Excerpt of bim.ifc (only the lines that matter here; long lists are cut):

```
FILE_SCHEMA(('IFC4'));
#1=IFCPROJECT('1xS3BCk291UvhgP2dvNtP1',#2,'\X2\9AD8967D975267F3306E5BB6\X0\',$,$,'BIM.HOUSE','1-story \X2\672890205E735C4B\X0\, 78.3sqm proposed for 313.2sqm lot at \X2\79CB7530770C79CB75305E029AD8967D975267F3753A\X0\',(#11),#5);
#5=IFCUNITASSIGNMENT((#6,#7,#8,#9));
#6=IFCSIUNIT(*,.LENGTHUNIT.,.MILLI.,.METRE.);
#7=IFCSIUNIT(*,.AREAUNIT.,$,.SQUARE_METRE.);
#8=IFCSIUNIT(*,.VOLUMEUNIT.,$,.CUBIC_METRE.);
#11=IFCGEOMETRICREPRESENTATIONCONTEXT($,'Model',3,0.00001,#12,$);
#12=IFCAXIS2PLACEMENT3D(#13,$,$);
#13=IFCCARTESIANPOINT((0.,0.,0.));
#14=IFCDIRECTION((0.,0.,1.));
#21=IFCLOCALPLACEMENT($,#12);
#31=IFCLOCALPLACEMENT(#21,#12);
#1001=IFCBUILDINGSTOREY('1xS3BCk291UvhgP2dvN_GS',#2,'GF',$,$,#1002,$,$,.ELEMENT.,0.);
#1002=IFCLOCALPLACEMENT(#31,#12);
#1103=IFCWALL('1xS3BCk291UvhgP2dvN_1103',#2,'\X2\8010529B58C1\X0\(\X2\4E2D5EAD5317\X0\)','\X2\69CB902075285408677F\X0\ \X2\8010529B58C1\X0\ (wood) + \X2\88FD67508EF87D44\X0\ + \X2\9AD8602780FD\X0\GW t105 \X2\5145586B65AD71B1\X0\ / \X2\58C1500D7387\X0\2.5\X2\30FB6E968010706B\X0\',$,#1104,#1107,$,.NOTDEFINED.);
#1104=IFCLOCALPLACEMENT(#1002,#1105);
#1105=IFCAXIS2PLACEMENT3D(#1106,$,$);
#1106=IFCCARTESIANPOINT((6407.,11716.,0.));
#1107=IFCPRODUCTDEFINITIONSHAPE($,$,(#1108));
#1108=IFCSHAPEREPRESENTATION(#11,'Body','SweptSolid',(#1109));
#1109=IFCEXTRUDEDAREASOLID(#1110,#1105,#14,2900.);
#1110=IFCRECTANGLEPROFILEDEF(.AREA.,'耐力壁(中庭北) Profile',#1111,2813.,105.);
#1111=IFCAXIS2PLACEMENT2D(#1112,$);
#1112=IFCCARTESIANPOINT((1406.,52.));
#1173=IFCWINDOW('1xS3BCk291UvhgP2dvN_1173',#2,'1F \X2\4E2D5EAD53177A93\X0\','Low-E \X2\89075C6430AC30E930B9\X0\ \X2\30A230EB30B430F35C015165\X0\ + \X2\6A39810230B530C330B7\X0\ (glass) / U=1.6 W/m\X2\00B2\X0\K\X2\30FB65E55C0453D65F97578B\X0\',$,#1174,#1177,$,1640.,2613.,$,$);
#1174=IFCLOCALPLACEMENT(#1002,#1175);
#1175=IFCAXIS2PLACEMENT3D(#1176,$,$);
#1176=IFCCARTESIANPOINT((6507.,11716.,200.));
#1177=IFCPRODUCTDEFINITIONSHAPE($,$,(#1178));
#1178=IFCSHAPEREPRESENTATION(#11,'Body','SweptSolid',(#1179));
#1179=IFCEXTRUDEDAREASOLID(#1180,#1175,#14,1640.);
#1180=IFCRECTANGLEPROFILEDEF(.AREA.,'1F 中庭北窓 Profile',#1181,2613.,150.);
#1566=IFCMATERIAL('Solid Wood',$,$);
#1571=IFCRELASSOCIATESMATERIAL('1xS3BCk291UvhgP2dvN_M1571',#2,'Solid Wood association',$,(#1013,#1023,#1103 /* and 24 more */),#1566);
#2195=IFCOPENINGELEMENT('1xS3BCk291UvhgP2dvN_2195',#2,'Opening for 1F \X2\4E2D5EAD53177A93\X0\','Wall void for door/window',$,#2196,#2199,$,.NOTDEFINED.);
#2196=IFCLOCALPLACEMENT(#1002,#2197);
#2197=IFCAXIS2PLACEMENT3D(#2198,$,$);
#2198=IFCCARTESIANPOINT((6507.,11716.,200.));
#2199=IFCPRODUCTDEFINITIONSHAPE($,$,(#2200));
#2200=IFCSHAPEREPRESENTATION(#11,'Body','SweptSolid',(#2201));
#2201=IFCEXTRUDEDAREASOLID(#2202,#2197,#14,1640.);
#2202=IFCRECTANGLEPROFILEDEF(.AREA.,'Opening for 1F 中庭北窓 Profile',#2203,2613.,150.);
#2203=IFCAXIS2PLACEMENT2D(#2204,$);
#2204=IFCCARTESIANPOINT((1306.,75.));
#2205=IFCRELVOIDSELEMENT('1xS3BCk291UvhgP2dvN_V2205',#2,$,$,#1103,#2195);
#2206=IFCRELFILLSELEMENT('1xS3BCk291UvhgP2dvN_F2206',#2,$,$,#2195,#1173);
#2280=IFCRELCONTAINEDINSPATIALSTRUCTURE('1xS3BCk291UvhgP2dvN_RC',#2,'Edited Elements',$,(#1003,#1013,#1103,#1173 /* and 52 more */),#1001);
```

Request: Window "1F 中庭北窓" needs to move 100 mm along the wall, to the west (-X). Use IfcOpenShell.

```python
import ifcopenshell
import ifcopenshell.api.geometry
import ifcopenshell.util.placement
import ifcopenshell.util.unit

model = ifcopenshell.open("bim.ifc")
unit_scale = ifcopenshell.util.unit.calculate_unit_scale(model)

window = model.by_id(1173)
opening = window.FillsVoids[0].RelatingOpeningElement
wall = opening.VoidsElements[0].RelatingBuildingElement

wall_matrix = ifcopenshell.util.placement.get_local_placement(wall.ObjectPlacement)
shift = wall_matrix[:3, 0] * -0.1 / unit_scale
before = ifcopenshell.util.placement.get_local_placement(window.ObjectPlacement)[:3, 3].copy()

# The window is not placed relative to its opening, so move both.
for product in (opening, window):
    matrix = ifcopenshell.util.placement.get_local_placement(product.ObjectPlacement)
    matrix[:3, 3] += shift
    ifcopenshell.api.geometry.edit_object_placement(model, product=product, matrix=matrix, is_si=False)

after = ifcopenshell.util.placement.get_local_placement(window.ObjectPlacement)[:3, 3]
print("window moved by", (after - before).round(3) + 0.0)

model.write("bim_edited.ifc")
```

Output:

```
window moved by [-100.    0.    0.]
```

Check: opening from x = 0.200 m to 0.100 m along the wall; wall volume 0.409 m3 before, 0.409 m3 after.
